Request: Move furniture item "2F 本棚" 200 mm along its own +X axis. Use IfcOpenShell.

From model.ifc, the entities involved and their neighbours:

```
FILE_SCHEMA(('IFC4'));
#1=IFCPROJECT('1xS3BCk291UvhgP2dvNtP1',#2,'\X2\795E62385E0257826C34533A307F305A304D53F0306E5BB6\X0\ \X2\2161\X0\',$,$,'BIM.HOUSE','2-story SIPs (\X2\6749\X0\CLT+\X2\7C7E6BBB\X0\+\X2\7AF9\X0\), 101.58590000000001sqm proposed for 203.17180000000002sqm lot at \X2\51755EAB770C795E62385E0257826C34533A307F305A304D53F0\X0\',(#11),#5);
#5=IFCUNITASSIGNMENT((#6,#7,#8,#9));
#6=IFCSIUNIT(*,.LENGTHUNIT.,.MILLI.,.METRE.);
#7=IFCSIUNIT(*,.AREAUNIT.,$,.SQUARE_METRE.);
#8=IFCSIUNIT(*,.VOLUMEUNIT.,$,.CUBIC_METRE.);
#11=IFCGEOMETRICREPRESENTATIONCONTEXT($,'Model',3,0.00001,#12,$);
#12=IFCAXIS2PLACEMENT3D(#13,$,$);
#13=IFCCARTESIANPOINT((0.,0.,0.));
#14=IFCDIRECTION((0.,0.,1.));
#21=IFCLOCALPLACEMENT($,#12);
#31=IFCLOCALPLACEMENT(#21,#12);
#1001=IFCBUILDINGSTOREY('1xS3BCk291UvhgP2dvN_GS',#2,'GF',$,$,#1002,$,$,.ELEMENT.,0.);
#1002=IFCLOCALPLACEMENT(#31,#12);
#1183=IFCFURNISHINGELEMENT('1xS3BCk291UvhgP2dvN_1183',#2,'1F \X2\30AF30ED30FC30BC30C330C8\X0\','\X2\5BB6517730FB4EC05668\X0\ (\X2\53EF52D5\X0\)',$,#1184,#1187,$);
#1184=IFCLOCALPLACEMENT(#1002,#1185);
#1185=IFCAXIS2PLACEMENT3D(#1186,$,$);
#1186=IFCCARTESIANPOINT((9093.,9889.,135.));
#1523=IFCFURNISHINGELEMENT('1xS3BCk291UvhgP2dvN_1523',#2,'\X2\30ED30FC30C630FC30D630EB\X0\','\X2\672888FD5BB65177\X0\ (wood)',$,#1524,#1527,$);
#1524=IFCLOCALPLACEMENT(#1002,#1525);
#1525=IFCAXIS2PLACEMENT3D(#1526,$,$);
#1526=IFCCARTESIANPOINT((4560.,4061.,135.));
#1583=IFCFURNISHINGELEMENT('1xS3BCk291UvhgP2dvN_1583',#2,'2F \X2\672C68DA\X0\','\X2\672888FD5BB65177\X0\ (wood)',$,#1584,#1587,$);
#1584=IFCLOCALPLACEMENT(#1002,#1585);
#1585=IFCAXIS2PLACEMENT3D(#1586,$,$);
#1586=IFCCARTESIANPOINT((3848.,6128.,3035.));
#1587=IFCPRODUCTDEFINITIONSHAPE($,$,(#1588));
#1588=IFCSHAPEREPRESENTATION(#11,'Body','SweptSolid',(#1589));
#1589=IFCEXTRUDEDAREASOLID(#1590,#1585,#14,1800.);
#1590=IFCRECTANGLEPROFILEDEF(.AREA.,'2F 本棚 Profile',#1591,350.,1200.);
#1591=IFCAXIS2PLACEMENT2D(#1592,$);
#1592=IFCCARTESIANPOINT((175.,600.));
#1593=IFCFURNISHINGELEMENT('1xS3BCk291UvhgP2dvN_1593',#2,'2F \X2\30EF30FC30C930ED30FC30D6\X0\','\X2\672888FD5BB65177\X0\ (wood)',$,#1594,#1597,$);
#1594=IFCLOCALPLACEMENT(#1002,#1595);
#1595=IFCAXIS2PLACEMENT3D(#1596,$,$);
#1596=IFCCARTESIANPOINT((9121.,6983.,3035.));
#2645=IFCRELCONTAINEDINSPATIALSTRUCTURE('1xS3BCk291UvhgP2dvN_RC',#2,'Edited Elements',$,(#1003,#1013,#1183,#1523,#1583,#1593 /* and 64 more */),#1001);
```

```python
import ifcopenshell
import ifcopenshell.api.geometry
import ifcopenshell.util.placement
import ifcopenshell.util.unit

model = ifcopenshell.open("model.ifc")
unit_scale = ifcopenshell.util.unit.calculate_unit_scale(model)

item = model.by_guid("1xS3BCk291UvhgP2dvN_1583")
matrix = ifcopenshell.util.placement.get_local_placement(item.ObjectPlacement)
matrix[:3, 3] += matrix[:3, 0] * 0.2 / unit_scale
ifcopenshell.api.geometry.edit_object_placement(model, product=item, matrix=matrix, is_si=False)

print(ifcopenshell.util.placement.get_local_placement(item.ObjectPlacement).round(3) + 0.0)

model.write("model_updated.ifc")
```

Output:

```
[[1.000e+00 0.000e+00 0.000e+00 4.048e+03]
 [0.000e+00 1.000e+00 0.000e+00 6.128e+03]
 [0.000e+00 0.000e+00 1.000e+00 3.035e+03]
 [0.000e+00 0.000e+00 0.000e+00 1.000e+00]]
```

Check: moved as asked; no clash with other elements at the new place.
